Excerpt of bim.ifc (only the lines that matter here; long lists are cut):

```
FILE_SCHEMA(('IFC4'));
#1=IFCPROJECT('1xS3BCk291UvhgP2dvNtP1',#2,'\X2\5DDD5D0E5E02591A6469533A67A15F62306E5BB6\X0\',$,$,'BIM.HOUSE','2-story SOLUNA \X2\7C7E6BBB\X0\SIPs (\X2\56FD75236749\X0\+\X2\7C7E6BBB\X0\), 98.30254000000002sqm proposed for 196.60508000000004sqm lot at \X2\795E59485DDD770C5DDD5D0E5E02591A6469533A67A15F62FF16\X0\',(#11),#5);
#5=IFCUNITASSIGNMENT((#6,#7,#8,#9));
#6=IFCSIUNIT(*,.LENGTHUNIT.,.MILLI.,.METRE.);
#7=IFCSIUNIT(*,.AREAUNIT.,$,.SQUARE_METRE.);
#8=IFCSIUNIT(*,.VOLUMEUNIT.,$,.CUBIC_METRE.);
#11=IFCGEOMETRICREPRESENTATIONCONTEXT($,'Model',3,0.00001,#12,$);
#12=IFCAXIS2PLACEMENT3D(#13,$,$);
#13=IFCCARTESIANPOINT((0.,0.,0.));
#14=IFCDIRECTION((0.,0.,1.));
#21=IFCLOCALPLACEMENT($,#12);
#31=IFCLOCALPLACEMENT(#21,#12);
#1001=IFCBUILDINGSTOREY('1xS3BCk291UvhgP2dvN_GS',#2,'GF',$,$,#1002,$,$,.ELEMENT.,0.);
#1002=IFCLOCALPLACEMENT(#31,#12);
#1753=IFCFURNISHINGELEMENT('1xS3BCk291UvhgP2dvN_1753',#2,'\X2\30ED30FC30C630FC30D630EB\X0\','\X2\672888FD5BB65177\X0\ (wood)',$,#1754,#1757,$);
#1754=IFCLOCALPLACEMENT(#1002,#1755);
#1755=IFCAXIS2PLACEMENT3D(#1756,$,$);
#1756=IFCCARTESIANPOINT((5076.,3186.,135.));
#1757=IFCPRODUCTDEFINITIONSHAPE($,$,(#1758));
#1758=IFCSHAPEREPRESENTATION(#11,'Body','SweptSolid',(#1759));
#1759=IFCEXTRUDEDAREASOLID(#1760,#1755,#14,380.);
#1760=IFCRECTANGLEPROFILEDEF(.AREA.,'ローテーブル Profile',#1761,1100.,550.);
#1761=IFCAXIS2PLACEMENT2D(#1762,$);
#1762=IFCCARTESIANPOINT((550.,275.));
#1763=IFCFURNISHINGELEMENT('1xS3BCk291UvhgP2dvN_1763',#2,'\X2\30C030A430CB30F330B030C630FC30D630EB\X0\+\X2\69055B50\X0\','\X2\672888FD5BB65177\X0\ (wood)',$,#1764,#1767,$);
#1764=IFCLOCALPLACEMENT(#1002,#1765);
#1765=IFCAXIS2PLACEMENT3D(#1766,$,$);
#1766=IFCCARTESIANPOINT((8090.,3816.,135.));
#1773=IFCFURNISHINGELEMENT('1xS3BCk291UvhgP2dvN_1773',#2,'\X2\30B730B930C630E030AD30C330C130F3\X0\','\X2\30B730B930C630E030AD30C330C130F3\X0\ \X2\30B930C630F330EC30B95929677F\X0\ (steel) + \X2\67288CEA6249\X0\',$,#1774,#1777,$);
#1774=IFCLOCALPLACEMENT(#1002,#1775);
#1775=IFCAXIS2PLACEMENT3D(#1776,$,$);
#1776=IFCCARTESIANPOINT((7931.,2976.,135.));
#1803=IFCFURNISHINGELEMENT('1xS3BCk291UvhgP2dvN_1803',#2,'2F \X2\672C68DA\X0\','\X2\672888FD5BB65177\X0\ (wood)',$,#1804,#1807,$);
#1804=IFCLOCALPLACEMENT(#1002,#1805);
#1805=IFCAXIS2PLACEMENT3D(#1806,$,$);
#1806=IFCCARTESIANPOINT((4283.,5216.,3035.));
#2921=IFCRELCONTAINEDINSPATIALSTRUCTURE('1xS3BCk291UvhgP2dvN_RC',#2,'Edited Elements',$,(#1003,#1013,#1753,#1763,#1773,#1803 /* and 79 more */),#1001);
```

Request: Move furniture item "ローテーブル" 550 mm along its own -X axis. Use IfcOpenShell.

```python
import ifcopenshell
import ifcopenshell.api.geometry
import ifcopenshell.util.placement

model = ifcopenshell.open("bim.ifc")

item = model.by_id(1753)
matrix = ifcopenshell.util.placement.get_local_placement(item.ObjectPlacement)
matrix[:3, 3] -= matrix[:3, 0] * 550.0
ifcopenshell.api.geometry.edit_object_placement(model, product=item, matrix=matrix, is_si=False)

print(ifcopenshell.util.placement.get_local_placement(item.ObjectPlacement).round(3) + 0.0)

model.write("bim_rev.ifc")
```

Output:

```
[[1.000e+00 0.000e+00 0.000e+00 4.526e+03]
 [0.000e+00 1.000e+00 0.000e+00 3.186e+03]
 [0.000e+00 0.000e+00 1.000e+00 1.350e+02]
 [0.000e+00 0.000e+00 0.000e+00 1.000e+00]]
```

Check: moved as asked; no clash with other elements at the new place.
